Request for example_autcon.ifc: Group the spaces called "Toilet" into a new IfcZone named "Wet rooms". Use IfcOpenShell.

First a look at what the model holds.

```python
import ifcopenshell

model = ifcopenshell.open("example_autcon.ifc")
print(model.schema)
seen = {}
for space in model.by_type("IfcSpace"):
    seen[space.LongName] = seen.get(space.LongName, 0) + 1
for name, count in sorted(seen.items(), key=str):
    print(count, "x", name)
print("zones:", [z.Name for z in model.by_type("IfcZone")][:20])
```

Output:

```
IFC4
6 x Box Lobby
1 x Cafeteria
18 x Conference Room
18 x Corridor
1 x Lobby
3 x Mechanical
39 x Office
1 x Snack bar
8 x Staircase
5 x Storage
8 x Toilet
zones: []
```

```python
import ifcopenshell
import ifcopenshell.api.group
import ifcopenshell.api.root

model = ifcopenshell.open("example_autcon.ifc")

names = {"Toilet"}
spaces = [s for s in model.by_type("IfcSpace") if s.LongName in names]

zone = ifcopenshell.api.root.create_entity(model, ifc_class="IfcZone", name="Wet rooms")
ifcopenshell.api.group.assign_group(model, products=spaces, group=zone)
print(len(spaces), "spaces in", zone.Name)

model.write("example_autcon_edited.ifc")
```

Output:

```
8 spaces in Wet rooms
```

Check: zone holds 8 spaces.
